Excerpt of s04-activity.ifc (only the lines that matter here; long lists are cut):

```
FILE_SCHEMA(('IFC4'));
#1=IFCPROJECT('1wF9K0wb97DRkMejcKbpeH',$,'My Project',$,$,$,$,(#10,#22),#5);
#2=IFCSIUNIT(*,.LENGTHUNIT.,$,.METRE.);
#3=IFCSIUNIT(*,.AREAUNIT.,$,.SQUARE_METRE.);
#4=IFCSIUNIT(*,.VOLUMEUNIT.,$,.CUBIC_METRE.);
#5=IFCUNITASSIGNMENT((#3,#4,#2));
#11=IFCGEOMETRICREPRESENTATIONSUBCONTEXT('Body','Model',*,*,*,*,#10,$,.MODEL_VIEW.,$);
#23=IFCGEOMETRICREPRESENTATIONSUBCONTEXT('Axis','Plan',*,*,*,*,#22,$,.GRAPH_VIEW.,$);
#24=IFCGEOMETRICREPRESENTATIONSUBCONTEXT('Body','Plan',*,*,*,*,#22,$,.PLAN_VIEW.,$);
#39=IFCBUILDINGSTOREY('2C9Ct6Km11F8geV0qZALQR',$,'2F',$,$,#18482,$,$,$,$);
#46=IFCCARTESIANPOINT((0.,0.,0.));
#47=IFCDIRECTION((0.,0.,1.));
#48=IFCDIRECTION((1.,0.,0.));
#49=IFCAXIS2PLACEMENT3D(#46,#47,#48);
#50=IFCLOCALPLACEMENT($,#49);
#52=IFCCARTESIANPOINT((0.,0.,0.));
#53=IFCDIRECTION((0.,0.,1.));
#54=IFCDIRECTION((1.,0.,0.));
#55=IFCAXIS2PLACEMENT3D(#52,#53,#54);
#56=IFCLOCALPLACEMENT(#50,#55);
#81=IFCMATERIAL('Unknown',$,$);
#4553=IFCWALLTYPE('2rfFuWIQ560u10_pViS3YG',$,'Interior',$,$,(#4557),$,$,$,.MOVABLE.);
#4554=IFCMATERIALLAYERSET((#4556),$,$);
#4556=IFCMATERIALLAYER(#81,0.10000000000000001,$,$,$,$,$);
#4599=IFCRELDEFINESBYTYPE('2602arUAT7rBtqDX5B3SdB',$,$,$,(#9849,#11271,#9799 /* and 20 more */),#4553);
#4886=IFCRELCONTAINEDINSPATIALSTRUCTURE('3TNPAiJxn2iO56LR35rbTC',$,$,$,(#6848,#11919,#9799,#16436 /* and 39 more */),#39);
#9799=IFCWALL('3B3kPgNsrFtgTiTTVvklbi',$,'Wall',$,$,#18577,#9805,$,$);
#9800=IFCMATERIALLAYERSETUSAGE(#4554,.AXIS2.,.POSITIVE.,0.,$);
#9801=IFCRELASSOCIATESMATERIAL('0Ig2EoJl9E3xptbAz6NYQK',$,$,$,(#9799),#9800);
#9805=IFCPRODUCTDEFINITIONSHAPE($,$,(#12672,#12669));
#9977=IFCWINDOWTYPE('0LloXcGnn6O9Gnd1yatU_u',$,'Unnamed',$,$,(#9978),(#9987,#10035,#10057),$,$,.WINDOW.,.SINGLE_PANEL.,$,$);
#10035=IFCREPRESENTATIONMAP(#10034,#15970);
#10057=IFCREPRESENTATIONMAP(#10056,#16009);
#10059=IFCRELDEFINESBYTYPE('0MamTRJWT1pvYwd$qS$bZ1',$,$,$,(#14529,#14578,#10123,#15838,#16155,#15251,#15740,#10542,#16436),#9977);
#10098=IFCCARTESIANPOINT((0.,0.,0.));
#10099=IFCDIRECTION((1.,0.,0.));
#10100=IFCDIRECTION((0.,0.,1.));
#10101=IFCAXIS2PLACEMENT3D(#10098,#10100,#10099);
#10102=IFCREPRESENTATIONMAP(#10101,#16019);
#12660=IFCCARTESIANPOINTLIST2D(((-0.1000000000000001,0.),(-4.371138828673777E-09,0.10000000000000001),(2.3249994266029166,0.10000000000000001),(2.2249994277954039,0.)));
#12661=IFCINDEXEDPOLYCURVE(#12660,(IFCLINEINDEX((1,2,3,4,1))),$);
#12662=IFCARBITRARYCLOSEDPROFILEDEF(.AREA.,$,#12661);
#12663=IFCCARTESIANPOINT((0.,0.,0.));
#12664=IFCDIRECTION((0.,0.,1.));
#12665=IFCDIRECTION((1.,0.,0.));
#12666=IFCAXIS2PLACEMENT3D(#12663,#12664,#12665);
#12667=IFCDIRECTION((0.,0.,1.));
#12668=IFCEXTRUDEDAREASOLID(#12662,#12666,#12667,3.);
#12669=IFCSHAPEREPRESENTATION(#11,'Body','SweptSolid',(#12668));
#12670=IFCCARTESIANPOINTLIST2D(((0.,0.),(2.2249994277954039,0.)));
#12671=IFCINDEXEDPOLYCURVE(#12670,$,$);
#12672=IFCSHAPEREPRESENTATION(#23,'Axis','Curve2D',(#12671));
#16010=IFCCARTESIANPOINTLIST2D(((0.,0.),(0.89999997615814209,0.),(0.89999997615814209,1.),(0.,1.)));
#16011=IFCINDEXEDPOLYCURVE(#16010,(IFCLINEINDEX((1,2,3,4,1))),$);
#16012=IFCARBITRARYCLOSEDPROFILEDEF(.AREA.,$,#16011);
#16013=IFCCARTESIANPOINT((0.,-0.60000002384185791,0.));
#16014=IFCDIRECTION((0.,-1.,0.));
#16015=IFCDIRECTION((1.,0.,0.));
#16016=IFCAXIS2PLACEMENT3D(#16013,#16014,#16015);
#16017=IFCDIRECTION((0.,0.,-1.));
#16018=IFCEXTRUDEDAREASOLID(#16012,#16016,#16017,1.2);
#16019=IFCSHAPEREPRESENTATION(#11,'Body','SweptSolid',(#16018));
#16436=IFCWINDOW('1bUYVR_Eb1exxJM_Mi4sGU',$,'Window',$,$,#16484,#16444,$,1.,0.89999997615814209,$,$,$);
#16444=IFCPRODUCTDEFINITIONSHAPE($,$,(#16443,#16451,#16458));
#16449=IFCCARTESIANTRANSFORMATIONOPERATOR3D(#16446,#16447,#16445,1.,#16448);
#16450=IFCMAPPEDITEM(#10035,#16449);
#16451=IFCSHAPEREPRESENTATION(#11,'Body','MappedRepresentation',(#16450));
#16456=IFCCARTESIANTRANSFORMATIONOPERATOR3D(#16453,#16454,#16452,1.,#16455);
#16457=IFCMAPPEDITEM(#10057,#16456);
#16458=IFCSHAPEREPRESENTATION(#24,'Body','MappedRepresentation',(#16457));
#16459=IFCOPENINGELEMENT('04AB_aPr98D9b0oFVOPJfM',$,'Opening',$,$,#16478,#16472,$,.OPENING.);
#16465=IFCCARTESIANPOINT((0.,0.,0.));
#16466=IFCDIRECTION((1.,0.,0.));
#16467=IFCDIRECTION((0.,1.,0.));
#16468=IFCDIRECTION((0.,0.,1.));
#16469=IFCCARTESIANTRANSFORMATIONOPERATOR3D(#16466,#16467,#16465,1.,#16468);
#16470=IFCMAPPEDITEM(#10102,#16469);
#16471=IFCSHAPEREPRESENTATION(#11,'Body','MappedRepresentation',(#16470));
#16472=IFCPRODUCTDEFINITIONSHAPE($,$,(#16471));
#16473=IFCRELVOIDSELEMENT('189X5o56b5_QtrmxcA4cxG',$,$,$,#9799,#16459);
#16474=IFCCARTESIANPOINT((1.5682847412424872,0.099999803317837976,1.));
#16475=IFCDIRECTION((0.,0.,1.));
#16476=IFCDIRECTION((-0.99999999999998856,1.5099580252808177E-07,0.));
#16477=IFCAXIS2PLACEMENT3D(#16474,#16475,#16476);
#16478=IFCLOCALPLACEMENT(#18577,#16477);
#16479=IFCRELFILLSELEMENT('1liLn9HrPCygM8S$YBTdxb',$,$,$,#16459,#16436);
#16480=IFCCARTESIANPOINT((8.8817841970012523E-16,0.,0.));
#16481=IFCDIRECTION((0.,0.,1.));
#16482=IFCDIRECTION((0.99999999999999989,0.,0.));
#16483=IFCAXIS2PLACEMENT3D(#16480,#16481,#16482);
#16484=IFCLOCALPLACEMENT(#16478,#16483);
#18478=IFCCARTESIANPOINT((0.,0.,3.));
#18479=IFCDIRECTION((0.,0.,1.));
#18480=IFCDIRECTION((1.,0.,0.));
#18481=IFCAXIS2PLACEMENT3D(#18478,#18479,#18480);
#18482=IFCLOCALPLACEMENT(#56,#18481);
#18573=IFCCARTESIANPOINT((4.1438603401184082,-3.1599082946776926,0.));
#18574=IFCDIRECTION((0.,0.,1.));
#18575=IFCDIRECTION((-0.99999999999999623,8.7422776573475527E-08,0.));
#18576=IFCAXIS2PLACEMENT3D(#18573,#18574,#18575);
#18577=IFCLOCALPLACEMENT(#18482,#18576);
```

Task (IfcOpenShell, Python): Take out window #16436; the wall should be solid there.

```python
import ifcopenshell
import ifcopenshell.api.feature
import ifcopenshell.api.root
import ifcopenshell.geom
import ifcopenshell.util.shape

model = ifcopenshell.open("s04-activity.ifc")
settings = ifcopenshell.geom.settings()


def volume(element):
    """Net volume in cubic metres, openings subtracted."""
    shape = ifcopenshell.geom.create_shape(settings, element)
    return ifcopenshell.util.shape.get_volume(shape.geometry)


window = model.by_id(16436)
opening = window.FillsVoids[0].RelatingOpeningElement
wall = opening.VoidsElements[0].RelatingBuildingElement
before = volume(wall)

ifcopenshell.api.root.remove_product(model, product=window)
ifcopenshell.api.feature.remove_feature(model, feature=opening)

after = volume(wall)

print(f"wall volume {before:.3f} -> {after:.3f} m3")

model.write("s04-activity_v2.ifc")
```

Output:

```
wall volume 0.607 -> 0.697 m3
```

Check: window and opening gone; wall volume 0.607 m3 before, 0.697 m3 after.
